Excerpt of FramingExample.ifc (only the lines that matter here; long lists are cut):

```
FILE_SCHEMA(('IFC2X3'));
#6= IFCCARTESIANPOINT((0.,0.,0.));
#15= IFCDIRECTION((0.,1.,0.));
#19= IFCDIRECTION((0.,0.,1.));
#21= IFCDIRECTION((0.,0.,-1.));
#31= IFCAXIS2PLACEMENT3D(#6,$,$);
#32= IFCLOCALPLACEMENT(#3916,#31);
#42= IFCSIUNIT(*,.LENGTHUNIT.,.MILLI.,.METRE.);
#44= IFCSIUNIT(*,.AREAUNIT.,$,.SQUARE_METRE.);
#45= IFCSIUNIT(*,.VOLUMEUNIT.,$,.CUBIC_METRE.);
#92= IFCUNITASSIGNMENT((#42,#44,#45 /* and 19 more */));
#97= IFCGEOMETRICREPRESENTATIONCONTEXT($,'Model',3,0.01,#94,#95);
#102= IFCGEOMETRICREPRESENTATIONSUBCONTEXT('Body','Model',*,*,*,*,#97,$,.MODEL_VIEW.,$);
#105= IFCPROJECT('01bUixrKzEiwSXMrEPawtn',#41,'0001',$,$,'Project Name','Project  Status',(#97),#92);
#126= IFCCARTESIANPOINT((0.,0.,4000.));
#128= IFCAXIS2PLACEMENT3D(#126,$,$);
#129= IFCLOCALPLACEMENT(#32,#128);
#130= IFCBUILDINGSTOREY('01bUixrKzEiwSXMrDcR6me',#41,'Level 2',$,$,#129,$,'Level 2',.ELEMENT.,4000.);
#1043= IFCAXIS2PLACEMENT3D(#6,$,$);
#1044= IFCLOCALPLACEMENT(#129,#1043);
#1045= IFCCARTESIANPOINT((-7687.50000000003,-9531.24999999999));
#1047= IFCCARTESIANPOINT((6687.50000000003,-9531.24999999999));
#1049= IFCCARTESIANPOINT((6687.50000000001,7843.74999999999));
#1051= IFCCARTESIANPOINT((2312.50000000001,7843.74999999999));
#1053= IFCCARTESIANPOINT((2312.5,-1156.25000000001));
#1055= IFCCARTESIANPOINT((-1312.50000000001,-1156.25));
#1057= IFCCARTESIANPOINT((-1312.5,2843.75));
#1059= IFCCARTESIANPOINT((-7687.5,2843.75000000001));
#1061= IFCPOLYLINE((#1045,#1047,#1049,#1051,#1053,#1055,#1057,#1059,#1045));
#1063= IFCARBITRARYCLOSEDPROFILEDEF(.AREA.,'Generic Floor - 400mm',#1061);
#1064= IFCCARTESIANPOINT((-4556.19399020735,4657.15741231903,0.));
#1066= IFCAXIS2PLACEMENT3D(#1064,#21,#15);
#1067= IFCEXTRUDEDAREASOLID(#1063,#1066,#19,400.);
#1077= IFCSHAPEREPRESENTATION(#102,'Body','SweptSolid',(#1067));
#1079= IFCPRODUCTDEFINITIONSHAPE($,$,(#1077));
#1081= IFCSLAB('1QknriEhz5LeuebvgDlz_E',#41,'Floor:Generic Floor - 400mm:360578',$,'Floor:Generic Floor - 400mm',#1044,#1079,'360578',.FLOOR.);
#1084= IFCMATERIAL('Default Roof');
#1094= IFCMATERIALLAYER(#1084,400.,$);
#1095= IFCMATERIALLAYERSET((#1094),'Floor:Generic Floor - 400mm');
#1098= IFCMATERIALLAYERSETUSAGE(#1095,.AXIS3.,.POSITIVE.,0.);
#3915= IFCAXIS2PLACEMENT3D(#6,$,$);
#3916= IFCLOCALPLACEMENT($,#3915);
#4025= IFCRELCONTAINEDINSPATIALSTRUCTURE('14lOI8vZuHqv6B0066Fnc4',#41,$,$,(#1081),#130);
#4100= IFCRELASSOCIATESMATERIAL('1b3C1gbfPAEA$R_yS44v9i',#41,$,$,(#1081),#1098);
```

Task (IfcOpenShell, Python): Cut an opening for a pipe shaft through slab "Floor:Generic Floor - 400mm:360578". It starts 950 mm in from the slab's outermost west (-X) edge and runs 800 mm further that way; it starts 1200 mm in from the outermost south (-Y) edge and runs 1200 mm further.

```python
import numpy as np
import ifcopenshell
import ifcopenshell.api.feature
import ifcopenshell.api.geometry
import ifcopenshell.api.root
import ifcopenshell.geom
import ifcopenshell.util.placement
import ifcopenshell.util.representation
import ifcopenshell.util.shape
import ifcopenshell.util.unit

model = ifcopenshell.open("FramingExample.ifc")
unit_scale = ifcopenshell.util.unit.calculate_unit_scale(model)
settings = ifcopenshell.geom.settings()


def volume(element):
    """Net volume in cubic metres, openings subtracted."""
    shape = ifcopenshell.geom.create_shape(settings, element)
    return ifcopenshell.util.shape.get_volume(shape.geometry)


slab = model.by_guid("1QknriEhz5LeuebvgDlz_E")
before = volume(slab)

# Extent in the slab's own axes, in metres. The edges named are its -X and -Y sides.
slab_shape = ifcopenshell.geom.create_shape(settings, slab)
vertices = ifcopenshell.util.shape.get_vertices(slab_shape.geometry)
x_min, y_min, bottom = vertices.min(axis=0)
top = vertices[:, 2].max()

opening = ifcopenshell.api.root.create_entity(model, ifc_class="IfcOpeningElement", name="Pipe shaft opening")
context = ifcopenshell.util.representation.get_context(model, "Model", "Body", "MODEL_VIEW")
width, depth = 0.8, 1.2
outline = [(0.0, 0.0), (width, 0.0), (width, depth), (0.0, depth), (0.0, 0.0)]
# Overshoot both faces by 50 mm so the cut is clean.
shape = ifcopenshell.api.geometry.add_slab_representation(
    model, context=context, depth=top - bottom + 0.1, polyline=outline
)
ifcopenshell.api.geometry.assign_representation(model, product=opening, representation=shape)

matrix = ifcopenshell.util.placement.get_local_placement(slab.ObjectPlacement)
matrix[:, 3] = matrix @ np.append(np.array([x_min + 0.95, y_min + 1.2, bottom - 0.05]) / unit_scale, 1.0)
ifcopenshell.api.geometry.edit_object_placement(model, product=opening, matrix=matrix, is_si=False)
ifcopenshell.api.feature.add_feature(model, feature=opening, element=slab)

after = volume(slab)

print(f"slab volume {before:.3f} -> {after:.3f} m3")

model.write("FramingExample_edited.ifc")
```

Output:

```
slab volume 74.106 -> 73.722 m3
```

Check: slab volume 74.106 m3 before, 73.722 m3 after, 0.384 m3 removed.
